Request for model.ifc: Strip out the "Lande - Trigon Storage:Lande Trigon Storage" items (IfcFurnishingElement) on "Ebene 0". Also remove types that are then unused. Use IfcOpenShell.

First a look at what the model holds.

```python
import ifcopenshell
import ifcopenshell.util.element

model = ifcopenshell.open("model.ifc")
print(model.schema)
storey = next(s for s in model.by_type("IfcBuildingStorey") if s.Name == "Ebene 0")
furniture = [e for e in ifcopenshell.util.element.get_decomposition(storey) if e.is_a("IfcFurnishingElement")]
seen = {}
for e in furniture:
    element_type = ifcopenshell.util.element.get_type(e)
    name = element_type.Name if element_type not in (None, e) else None
    seen[name] = seen.get(name, 0) + 1
for name, count in sorted(seen.items(), key=str):
    print(count, "x", name)
```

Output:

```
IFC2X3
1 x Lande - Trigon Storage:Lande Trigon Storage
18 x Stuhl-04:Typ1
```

```python
import ifcopenshell
import ifcopenshell.api.root
import ifcopenshell.util.element

model = ifcopenshell.open("model.ifc")

storey = next(s for s in model.by_type("IfcBuildingStorey") if s.Name == "Ebene 0")
furniture = [e for e in ifcopenshell.util.element.get_decomposition(storey) if e.is_a("IfcFurnishingElement")]
targets = [e for e in furniture if (t := ifcopenshell.util.element.get_type(e)) not in (None, e) and t.Name == "Lande - Trigon Storage:Lande Trigon Storage"]
types = {ifcopenshell.util.element.get_type(e) for e in targets} - {None, *targets}

for e in targets:
    ifcopenshell.api.root.remove_product(model, product=e)
print(len(targets), "removed")

unused = [t for t in types if not ifcopenshell.util.element.get_types(t)]
for t in unused:
    ifcopenshell.api.root.remove_product(model, product=t)
print(len(unused), "unused types removed")

model.write("model_edited.ifc")
```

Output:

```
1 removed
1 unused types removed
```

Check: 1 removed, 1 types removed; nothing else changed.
